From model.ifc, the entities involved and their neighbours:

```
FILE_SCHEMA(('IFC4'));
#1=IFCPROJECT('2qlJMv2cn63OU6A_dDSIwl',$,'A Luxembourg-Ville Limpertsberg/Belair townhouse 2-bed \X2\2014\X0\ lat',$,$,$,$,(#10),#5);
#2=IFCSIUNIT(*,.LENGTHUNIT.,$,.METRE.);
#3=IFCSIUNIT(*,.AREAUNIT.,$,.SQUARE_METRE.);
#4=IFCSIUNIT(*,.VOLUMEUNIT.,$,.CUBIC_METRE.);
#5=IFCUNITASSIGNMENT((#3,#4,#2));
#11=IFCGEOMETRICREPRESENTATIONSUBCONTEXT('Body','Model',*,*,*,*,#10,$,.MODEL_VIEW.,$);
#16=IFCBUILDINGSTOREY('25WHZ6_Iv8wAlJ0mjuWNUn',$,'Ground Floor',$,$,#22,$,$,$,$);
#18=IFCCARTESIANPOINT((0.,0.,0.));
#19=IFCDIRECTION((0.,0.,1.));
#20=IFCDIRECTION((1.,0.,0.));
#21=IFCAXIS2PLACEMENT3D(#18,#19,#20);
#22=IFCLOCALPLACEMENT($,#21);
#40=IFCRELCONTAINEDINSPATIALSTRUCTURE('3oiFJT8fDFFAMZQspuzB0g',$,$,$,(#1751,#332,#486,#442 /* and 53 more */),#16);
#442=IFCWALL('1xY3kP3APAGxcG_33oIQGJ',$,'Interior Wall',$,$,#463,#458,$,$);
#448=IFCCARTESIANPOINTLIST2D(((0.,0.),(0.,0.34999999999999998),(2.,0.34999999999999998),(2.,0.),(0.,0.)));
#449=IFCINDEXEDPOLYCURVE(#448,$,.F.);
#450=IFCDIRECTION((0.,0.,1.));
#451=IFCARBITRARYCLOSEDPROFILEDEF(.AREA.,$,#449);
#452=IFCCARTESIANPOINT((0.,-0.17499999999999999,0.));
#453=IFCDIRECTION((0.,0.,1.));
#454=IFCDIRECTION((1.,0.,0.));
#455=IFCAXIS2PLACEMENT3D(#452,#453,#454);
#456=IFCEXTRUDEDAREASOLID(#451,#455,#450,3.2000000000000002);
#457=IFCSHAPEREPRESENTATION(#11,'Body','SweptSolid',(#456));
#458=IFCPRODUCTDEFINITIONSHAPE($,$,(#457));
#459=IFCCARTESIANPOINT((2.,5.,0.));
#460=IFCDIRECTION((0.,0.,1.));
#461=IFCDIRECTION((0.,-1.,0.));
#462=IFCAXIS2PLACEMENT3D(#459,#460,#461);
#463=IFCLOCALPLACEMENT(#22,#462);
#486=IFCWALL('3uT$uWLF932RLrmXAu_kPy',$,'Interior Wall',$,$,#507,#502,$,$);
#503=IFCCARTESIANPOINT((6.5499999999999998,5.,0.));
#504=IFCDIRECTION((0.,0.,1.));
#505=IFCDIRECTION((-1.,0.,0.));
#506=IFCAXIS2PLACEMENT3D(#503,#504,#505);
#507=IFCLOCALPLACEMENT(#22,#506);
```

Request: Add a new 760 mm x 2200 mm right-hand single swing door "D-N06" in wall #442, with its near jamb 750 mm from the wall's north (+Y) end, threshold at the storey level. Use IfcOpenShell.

```python
import numpy as np
import ifcopenshell
import ifcopenshell.api.feature
import ifcopenshell.api.geometry
import ifcopenshell.api.root
import ifcopenshell.api.spatial
import ifcopenshell.geom
import ifcopenshell.util.element
import ifcopenshell.util.placement
import ifcopenshell.util.representation
import ifcopenshell.util.shape
import ifcopenshell.util.unit

model = ifcopenshell.open("model.ifc")
unit_scale = ifcopenshell.util.unit.calculate_unit_scale(model)
settings = ifcopenshell.geom.settings()


def volume(element):
    """Net volume in cubic metres, openings subtracted."""
    shape = ifcopenshell.geom.create_shape(settings, element)
    return ifcopenshell.util.shape.get_volume(shape.geometry)


wall = model.by_guid("1xY3kP3APAGxcG_33oIQGJ")
storey = ifcopenshell.util.element.get_container(wall, ifc_class="IfcBuildingStorey")
context = ifcopenshell.util.representation.get_context(model, "Model", "Body", "MODEL_VIEW")
before = volume(wall)

width, height, from_end, sill = 0.76, 2.2, 0.75, 0.0  # metres

# The wall runs along its own X axis, and the end named is its -X end.
wall_shape = ifcopenshell.geom.create_shape(settings, wall)
x, y, z = ifcopenshell.util.shape.get_vertices(wall_shape.geometry).T
start = x.min() + from_end
face, thickness = float(y.min()), float(y.max() - y.min())
wall_matrix = ifcopenshell.util.placement.get_local_placement(wall.ObjectPlacement)
level = ifcopenshell.util.placement.get_local_placement(storey.ObjectPlacement)[2, 3]


def in_wall(x, y):
    """Placement at x, y metres in the wall's axes, at sill height."""
    matrix = wall_matrix.copy()
    matrix[:, 3] = wall_matrix @ np.array([x / unit_scale, y / unit_scale, 0.0, 1.0])
    matrix[2, 3] = level + sill / unit_scale
    return matrix


# Opening: a box that overshoots both wall faces by 50 mm.
opening = ifcopenshell.api.root.create_entity(model, ifc_class="IfcOpeningElement", predefined_type="OPENING")
box = ifcopenshell.api.geometry.add_wall_representation(
    model, context=context, length=width, height=height, thickness=thickness + 0.1
)
ifcopenshell.api.geometry.assign_representation(model, product=opening, representation=box)
ifcopenshell.api.geometry.edit_object_placement(model, product=opening, matrix=in_wall(start, face - 0.05), is_si=False)
ifcopenshell.api.feature.add_feature(model, feature=opening, element=wall)

door = ifcopenshell.api.root.create_entity(model, ifc_class="IfcDoor", name="D-N06", predefined_type="DOOR")
door.OverallWidth, door.OverallHeight = width / unit_scale, height / unit_scale
door.OperationType = "SINGLE_SWING_RIGHT"
body = ifcopenshell.api.geometry.add_door_representation(
    model,
    context=context,
    overall_width=door.OverallWidth,
    overall_height=door.OverallHeight,
    operation_type="SINGLE_SWING_RIGHT",
    lining_properties={"LiningDepth": thickness / unit_scale, "ThresholdDepth": thickness / unit_scale},
)
ifcopenshell.api.geometry.assign_representation(model, product=door, representation=body)
ifcopenshell.api.spatial.assign_container(model, products=[door], relating_structure=storey)
ifcopenshell.api.feature.add_filling(model, opening=opening, element=door)

# The lining spans the wall, so the door starts at the wall face.
ifcopenshell.api.geometry.edit_object_placement(model, product=door, matrix=in_wall(start, face), is_si=False)

after = volume(wall)

print(f"wall volume {before:.3f} -> {after:.3f} m3")

model.write("model_rev.ifc")
```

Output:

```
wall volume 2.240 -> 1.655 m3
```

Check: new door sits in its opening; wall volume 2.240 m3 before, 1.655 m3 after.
